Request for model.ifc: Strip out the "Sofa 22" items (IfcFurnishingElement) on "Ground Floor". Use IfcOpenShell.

First a look at what the model holds.

```python
import ifcopenshell
import ifcopenshell.util.element

model = ifcopenshell.open("model.ifc")
print(model.schema)
storey = next(s for s in model.by_type("IfcBuildingStorey") if s.Name == "Ground Floor")
furniture = [e for e in ifcopenshell.util.element.get_decomposition(storey) if e.is_a("IfcFurnishingElement")]
seen = {}
for e in furniture:
    element_type = ifcopenshell.util.element.get_type(e)
    name = element_type.Name if element_type not in (None, e) else None
    seen[name] = seen.get(name, 0) + 1
for name, count in sorted(seen.items(), key=str):
    print(count, "x", name)
```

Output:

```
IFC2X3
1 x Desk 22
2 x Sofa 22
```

```python
import ifcopenshell
import ifcopenshell.api.root
import ifcopenshell.util.element

model = ifcopenshell.open("model.ifc")

storey = next(s for s in model.by_type("IfcBuildingStorey") if s.Name == "Ground Floor")
furniture = [e for e in ifcopenshell.util.element.get_decomposition(storey) if e.is_a("IfcFurnishingElement")]
targets = [e for e in furniture if (t := ifcopenshell.util.element.get_type(e)) not in (None, e) and t.Name == "Sofa 22"]

for e in targets:
    ifcopenshell.api.root.remove_product(model, product=e)
print(len(targets), "removed")

model.write("model_v2.ifc")
```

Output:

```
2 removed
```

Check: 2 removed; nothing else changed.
